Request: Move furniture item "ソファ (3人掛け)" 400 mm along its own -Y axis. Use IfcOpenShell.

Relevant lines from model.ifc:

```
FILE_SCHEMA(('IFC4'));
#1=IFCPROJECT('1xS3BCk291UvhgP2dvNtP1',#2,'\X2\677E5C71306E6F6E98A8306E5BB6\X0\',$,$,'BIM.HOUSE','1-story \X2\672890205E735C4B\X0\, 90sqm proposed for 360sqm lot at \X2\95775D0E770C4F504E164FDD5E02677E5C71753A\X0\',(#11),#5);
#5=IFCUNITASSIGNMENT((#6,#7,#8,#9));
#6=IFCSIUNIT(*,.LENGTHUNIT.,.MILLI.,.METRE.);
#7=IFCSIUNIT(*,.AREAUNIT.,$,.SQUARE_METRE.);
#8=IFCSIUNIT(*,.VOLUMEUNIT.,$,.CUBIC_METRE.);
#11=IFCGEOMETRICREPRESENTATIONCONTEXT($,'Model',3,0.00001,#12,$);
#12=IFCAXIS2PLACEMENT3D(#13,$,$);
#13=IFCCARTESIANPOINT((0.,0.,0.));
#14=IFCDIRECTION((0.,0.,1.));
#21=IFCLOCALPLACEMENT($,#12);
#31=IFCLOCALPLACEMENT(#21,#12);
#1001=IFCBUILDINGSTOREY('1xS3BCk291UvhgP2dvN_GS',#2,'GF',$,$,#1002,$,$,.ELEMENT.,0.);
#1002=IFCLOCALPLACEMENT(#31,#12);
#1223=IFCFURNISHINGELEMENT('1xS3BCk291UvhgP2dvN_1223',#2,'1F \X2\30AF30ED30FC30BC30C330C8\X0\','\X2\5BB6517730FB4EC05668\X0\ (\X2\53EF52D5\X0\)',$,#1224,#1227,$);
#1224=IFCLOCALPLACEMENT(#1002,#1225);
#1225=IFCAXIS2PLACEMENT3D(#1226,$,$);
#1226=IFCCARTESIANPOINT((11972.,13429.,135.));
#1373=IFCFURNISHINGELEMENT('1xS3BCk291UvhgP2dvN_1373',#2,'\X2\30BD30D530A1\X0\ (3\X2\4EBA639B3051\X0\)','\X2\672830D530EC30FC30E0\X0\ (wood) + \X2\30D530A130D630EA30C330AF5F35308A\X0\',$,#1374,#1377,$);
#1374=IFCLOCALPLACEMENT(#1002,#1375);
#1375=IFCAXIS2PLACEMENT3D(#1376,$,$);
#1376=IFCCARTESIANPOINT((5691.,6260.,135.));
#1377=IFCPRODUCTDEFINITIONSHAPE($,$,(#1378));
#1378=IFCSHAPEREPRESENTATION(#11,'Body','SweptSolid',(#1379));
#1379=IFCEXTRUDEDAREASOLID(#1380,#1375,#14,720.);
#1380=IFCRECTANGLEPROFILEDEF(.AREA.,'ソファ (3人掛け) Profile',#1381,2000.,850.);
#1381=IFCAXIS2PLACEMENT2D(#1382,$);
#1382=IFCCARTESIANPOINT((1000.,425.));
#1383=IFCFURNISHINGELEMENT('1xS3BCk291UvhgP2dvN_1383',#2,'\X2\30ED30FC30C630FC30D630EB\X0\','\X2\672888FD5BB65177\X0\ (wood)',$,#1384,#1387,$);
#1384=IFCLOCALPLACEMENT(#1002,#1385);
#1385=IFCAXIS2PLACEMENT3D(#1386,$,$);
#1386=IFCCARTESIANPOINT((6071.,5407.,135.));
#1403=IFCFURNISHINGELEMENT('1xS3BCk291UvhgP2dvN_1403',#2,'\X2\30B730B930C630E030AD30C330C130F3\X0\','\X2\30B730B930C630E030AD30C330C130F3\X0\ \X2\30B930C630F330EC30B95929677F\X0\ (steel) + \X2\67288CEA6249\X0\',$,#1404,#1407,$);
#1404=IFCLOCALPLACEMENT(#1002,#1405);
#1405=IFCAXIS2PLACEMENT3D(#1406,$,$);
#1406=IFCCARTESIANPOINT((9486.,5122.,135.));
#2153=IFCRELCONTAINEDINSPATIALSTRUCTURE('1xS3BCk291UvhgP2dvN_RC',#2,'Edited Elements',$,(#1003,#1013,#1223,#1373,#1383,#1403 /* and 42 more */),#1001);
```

```python
import ifcopenshell
import ifcopenshell.api.geometry
import ifcopenshell.util.placement
import ifcopenshell.util.unit

model = ifcopenshell.open("model.ifc")
unit_scale = ifcopenshell.util.unit.calculate_unit_scale(model)

item = model.by_guid("1xS3BCk291UvhgP2dvN_1373")
matrix = ifcopenshell.util.placement.get_local_placement(item.ObjectPlacement)
matrix[:3, 3] -= matrix[:3, 1] * 0.4 / unit_scale
ifcopenshell.api.geometry.edit_object_placement(model, product=item, matrix=matrix, is_si=False)

print(ifcopenshell.util.placement.get_local_placement(item.ObjectPlacement).round(3) + 0.0)

model.write("model_rev.ifc")
```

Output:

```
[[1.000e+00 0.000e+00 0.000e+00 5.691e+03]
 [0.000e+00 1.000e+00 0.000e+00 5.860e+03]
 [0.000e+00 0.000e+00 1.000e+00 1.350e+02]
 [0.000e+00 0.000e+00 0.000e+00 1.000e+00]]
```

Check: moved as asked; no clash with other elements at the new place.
